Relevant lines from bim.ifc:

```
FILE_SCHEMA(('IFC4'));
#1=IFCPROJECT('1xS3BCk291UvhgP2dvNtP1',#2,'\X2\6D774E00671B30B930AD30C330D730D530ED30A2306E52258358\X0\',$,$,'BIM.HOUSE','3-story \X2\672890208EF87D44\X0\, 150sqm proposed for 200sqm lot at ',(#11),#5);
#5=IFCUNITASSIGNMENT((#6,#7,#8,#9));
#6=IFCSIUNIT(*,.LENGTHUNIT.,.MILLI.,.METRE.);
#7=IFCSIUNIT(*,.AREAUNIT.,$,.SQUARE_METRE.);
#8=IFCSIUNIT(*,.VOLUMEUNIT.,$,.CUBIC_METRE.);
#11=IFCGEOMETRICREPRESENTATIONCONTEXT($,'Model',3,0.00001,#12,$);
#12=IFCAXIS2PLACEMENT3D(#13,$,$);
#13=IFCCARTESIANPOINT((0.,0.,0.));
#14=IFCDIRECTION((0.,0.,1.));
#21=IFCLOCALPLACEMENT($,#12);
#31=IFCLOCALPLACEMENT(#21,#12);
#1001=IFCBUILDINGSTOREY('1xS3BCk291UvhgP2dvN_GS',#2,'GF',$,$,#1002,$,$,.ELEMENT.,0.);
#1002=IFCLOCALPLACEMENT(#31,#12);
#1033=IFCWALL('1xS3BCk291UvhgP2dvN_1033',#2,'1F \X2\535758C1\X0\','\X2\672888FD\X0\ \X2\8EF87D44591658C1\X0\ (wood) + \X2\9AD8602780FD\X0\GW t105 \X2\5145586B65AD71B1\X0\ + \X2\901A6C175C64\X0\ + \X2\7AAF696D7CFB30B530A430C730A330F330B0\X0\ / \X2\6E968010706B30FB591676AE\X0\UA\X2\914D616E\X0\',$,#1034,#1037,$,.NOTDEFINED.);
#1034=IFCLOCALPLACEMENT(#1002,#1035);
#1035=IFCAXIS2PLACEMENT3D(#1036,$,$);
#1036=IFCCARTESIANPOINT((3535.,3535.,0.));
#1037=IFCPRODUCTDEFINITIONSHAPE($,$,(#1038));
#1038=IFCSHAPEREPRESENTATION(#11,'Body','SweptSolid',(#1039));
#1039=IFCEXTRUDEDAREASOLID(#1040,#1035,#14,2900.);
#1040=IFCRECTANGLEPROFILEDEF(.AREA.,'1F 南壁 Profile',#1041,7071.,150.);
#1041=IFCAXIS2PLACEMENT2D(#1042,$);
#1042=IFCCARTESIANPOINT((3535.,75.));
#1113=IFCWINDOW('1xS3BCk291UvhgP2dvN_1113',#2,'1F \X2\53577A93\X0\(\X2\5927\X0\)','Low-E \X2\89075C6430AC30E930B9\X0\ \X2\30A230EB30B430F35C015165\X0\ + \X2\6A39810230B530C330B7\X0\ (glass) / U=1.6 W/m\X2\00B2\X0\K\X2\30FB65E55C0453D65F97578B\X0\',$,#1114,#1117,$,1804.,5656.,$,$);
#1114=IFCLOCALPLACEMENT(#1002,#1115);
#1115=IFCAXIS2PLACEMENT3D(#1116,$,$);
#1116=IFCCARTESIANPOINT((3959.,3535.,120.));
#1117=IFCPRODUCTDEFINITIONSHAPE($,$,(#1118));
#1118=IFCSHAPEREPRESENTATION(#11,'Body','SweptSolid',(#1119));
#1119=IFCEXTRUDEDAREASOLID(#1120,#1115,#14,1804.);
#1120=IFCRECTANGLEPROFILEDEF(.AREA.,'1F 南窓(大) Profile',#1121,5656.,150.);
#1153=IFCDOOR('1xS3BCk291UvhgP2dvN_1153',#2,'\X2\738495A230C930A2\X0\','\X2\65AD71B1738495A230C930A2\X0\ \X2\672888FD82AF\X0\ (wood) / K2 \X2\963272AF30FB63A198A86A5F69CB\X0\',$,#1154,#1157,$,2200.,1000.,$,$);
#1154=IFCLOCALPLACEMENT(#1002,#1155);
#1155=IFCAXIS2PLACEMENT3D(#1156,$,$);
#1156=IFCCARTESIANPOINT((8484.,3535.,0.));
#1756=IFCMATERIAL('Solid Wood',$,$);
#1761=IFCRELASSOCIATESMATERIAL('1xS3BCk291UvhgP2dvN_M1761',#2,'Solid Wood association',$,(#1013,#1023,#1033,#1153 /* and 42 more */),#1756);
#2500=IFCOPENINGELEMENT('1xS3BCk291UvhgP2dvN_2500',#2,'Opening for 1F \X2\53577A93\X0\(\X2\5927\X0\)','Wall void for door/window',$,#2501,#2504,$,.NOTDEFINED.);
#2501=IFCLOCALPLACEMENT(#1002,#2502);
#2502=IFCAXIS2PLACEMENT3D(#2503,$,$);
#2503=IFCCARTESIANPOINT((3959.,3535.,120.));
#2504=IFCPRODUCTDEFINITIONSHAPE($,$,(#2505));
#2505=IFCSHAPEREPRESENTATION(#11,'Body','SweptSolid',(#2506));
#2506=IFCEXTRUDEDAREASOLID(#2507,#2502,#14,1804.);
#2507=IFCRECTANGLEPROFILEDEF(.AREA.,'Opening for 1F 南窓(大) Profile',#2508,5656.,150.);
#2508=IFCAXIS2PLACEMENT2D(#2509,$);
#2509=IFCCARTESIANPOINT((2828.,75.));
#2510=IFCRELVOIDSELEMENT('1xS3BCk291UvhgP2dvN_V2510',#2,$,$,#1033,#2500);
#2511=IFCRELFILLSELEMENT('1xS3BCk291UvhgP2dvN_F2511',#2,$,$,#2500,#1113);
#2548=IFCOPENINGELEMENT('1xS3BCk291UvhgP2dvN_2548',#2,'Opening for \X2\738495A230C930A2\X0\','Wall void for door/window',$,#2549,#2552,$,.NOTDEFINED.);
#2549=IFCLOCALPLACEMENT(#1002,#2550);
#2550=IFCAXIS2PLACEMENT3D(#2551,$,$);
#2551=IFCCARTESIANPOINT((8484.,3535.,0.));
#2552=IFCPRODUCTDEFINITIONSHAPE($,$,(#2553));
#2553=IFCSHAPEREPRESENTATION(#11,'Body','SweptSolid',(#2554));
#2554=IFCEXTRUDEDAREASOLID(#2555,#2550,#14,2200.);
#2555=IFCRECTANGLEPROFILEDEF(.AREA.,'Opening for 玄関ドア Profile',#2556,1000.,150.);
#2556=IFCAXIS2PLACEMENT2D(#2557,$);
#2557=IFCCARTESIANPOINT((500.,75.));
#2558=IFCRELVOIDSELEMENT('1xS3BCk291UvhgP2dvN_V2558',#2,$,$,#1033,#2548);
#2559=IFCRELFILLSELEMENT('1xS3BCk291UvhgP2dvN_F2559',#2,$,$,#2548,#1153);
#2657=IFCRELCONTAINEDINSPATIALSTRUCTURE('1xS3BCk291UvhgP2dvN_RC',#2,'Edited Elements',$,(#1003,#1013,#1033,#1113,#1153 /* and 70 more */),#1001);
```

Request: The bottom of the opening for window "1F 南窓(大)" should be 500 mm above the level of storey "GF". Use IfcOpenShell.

```python
import numpy as np
import ifcopenshell
import ifcopenshell.api.geometry
import ifcopenshell.geom
import ifcopenshell.util.element
import ifcopenshell.util.placement
import ifcopenshell.util.shape
import ifcopenshell.util.unit

model = ifcopenshell.open("bim.ifc")
unit_scale = ifcopenshell.util.unit.calculate_unit_scale(model)

window = model.by_guid("1xS3BCk291UvhgP2dvN_1113")
opening = window.FillsVoids[0].RelatingOpeningElement
storey = ifcopenshell.util.element.get_container(window, ifc_class="IfcBuildingStorey")
level = ifcopenshell.util.placement.get_local_placement(storey.ObjectPlacement)[2, 3]

# The opening's origin need not be at the sill, so measure its lowest point.
shape = ifcopenshell.geom.create_shape(ifcopenshell.geom.settings(), opening)
bottom = ifcopenshell.util.shape.get_shape_bottom_elevation(shape, shape.geometry) / unit_scale
dz = level + 0.5 / unit_scale - bottom

shift = np.array([0.0, 0.0, dz])
# The window is not placed relative to its opening, so move both.
for product in (opening, window):
    matrix = ifcopenshell.util.placement.get_local_placement(product.ObjectPlacement)
    matrix[:3, 3] += shift
    ifcopenshell.api.geometry.edit_object_placement(model, product=product, matrix=matrix, is_si=False)

print(f"moved by {dz * unit_scale:+.3f} m")

model.write("bim_edited.ifc")
```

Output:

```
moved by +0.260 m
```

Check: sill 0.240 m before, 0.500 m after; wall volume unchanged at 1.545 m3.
